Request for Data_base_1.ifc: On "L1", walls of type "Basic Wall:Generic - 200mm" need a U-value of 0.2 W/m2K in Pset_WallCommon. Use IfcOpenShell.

First a look at what the model holds.

```python
import ifcopenshell
import ifcopenshell.util.element

model = ifcopenshell.open("Data_base_1.ifc")
print(model.schema)
storey = next(s for s in model.by_type("IfcBuildingStorey") if s.Name == "L1")
walls = [e for e in ifcopenshell.util.element.get_decomposition(storey) if e.is_a("IfcWall")]
seen = {}
for e in walls:
    element_type = ifcopenshell.util.element.get_type(e)
    key = (element_type.Name if element_type != e and element_type else None, ifcopenshell.util.element.get_pset(e, "Pset_WallCommon", "ThermalTransmittance"))
    seen[key] = seen.get(key, 0) + 1
for (name, value), count in sorted(seen.items(), key=str):
    print(count, "x", name, "|", value)
```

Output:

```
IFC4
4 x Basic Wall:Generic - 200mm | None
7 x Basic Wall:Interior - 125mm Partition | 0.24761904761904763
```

```python
import ifcopenshell
import ifcopenshell.api.pset
import ifcopenshell.util.element

model = ifcopenshell.open("Data_base_1.ifc")

storey = next(s for s in model.by_type("IfcBuildingStorey") if s.Name == "L1")
walls = [e for e in ifcopenshell.util.element.get_decomposition(storey) if e.is_a("IfcWall")]

count = 0
for e in walls:
    element_type = ifcopenshell.util.element.get_type(e)
    if element_type in (None, e) or element_type.Name != "Basic Wall:Generic - 200mm":
        continue
    # add_pset returns the element's existing set when there is one.
    pset = ifcopenshell.api.pset.add_pset(model, product=e, name="Pset_WallCommon")
    ifcopenshell.api.pset.edit_pset(model, pset=pset, properties={"ThermalTransmittance": 0.2})
    count += 1

print(count, "walls updated")

model.write("Data_base_1_rev.ifc")
```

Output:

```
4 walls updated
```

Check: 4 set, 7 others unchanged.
